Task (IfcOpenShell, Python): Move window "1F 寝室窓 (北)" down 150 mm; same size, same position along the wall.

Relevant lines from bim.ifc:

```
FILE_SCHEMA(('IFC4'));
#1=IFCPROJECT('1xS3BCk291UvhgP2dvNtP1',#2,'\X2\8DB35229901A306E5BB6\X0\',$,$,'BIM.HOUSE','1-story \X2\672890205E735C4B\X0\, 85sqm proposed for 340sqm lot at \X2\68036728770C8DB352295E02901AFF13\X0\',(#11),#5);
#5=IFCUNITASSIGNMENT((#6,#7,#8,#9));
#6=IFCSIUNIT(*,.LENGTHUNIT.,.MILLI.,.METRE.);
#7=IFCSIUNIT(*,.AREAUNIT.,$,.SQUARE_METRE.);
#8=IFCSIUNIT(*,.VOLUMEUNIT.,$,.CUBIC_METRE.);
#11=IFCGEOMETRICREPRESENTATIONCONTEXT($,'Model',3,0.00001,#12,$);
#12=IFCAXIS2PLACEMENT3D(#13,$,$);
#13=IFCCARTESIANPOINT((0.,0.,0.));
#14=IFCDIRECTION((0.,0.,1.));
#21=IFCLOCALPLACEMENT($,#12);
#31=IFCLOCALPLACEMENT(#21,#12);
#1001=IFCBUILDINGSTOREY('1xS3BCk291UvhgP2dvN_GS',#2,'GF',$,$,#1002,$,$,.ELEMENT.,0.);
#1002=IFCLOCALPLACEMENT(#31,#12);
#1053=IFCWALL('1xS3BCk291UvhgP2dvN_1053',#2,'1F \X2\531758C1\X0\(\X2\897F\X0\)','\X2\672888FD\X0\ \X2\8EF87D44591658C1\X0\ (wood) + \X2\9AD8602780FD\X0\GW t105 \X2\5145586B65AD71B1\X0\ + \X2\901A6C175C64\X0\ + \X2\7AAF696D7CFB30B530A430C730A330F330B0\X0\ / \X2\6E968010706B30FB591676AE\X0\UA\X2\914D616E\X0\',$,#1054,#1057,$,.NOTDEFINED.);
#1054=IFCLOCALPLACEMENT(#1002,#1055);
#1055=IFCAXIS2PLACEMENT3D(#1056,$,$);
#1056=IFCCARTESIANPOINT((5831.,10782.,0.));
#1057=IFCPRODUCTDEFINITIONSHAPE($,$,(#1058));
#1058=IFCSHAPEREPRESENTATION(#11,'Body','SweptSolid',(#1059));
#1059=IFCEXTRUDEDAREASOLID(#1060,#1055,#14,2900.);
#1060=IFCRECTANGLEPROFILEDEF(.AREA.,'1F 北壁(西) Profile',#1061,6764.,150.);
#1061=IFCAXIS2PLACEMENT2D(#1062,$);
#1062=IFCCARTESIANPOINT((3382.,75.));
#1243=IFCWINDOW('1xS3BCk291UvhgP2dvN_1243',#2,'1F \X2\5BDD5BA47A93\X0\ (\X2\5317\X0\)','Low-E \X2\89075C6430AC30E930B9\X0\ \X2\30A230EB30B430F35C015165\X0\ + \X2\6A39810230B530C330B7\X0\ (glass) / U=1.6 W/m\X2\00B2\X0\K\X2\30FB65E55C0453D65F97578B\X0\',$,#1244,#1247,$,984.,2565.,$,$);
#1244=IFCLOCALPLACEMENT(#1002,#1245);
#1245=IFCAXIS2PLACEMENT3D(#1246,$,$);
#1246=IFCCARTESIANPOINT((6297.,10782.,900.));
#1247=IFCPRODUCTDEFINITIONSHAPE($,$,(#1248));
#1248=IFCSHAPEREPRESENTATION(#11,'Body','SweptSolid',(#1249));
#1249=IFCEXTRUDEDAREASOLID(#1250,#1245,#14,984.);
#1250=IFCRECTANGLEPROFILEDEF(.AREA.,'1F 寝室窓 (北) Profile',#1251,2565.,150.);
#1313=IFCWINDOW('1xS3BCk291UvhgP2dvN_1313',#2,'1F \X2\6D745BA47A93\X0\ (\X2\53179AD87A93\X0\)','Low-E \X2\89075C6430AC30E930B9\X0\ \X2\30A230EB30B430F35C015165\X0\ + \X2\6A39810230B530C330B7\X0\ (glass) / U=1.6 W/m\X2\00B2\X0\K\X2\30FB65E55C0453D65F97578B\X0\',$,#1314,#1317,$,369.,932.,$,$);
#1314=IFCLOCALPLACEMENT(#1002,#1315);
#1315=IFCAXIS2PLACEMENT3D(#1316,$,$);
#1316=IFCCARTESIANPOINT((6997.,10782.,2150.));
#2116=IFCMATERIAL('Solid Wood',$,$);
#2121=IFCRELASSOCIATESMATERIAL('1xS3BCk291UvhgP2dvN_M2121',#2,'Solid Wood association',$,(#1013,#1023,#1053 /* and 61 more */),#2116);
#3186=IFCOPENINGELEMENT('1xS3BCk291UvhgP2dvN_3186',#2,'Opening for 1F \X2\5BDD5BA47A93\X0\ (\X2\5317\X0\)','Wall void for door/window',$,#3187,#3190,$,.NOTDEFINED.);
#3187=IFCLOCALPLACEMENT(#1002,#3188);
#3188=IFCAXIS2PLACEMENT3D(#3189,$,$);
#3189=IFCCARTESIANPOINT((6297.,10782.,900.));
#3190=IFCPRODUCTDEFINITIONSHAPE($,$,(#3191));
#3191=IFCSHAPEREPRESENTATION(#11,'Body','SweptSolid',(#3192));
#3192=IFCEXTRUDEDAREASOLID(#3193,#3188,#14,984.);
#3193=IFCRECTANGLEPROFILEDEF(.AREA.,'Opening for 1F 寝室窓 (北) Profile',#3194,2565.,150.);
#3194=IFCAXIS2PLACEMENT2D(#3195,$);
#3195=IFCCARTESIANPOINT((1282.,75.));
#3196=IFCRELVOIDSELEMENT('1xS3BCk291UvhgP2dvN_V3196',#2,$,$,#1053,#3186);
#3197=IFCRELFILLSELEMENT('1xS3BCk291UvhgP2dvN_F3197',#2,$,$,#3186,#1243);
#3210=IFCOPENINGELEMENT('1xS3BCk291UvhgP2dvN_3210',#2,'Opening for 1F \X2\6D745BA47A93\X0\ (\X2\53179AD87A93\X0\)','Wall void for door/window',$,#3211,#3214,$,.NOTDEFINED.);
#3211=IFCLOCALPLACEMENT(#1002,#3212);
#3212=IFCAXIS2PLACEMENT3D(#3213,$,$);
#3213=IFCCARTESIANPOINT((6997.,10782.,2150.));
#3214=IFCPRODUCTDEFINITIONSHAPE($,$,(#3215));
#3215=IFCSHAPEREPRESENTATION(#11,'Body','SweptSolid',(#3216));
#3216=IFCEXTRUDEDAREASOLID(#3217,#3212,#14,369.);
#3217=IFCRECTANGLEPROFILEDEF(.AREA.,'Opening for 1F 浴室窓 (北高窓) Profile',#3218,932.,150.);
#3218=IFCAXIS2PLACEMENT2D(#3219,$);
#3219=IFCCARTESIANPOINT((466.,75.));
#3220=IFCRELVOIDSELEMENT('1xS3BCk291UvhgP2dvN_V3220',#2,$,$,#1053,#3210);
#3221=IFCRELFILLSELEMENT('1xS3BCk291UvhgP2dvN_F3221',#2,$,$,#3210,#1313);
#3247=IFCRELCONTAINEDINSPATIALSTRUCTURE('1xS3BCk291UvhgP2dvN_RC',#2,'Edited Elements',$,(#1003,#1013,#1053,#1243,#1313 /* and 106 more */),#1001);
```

```python
import numpy as np
import ifcopenshell
import ifcopenshell.api.geometry
import ifcopenshell.util.placement
import ifcopenshell.util.unit

model = ifcopenshell.open("bim.ifc")
unit_scale = ifcopenshell.util.unit.calculate_unit_scale(model)

window = model.by_guid("1xS3BCk291UvhgP2dvN_1243")
opening = window.FillsVoids[0].RelatingOpeningElement
dz = -150.0

shift = np.array([0.0, 0.0, dz])
# The window is not placed relative to its opening, so move both.
for product in (opening, window):
    matrix = ifcopenshell.util.placement.get_local_placement(product.ObjectPlacement)
    matrix[:3, 3] += shift
    ifcopenshell.api.geometry.edit_object_placement(model, product=product, matrix=matrix, is_si=False)

print(f"moved by {dz * unit_scale:+.3f} m")

model.write("bim_updated.ifc")
```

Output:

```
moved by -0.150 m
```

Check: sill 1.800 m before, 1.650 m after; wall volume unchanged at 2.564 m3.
